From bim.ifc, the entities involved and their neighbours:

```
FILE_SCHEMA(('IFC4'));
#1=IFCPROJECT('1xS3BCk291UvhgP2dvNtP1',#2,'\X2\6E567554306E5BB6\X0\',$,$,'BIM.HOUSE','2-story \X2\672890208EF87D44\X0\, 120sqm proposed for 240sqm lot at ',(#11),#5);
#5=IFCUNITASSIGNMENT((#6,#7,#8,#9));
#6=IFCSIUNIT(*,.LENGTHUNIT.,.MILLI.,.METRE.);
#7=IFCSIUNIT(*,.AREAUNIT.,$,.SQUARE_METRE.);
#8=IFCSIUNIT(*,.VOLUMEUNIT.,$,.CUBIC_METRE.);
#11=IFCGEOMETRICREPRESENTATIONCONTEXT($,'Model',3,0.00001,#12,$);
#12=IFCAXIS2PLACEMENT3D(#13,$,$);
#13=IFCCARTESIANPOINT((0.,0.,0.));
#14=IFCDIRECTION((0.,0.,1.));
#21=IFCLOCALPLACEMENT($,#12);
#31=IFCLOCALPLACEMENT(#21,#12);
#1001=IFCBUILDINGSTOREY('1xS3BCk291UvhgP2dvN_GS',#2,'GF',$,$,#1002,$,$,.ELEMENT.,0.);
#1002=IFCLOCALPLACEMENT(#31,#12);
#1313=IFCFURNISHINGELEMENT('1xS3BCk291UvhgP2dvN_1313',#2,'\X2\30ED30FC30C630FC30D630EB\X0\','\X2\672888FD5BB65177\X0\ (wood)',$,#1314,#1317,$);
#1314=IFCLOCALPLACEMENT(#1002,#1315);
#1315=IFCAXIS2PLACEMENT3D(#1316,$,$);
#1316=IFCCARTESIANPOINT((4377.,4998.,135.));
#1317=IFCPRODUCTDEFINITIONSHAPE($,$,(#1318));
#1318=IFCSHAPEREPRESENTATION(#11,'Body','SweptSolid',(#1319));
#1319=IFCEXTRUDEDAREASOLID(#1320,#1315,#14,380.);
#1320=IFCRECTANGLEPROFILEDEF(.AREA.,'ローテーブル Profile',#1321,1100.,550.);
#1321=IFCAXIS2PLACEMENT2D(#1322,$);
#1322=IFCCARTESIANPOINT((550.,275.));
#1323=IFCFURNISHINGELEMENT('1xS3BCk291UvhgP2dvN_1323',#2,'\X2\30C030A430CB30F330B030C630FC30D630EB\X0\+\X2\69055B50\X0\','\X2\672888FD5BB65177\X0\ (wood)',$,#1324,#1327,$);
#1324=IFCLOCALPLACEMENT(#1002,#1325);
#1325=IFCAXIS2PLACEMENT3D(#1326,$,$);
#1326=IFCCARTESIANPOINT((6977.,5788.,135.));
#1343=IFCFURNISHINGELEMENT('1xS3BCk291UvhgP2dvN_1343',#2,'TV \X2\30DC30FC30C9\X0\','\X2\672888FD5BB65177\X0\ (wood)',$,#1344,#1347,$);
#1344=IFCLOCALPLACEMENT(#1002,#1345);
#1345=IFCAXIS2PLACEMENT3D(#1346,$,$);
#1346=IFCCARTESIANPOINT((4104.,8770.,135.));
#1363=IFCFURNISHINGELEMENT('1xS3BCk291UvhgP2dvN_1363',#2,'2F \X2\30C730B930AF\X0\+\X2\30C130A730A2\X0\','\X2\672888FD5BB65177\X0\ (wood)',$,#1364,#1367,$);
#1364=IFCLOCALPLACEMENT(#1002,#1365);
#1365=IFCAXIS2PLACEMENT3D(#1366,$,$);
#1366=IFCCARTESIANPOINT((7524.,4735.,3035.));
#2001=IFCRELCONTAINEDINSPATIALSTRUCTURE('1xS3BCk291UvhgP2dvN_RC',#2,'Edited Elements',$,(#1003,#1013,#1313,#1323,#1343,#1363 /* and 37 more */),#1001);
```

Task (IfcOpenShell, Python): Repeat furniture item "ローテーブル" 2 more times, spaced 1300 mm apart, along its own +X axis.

```python
import ifcopenshell
import ifcopenshell.api.geometry
import ifcopenshell.api.root
import ifcopenshell.util.element
import ifcopenshell.util.placement
import ifcopenshell.util.unit

model = ifcopenshell.open("bim.ifc")
unit_scale = ifcopenshell.util.unit.calculate_unit_scale(model)


def reuse_history(source, copy):
    """copy_class also copies each property set's owner history, people and application; keep the originals."""
    for rel in copy.IsDefinedBy:
        if rel.is_a("IfcRelDefinesByProperties") and (history := rel.RelatingPropertyDefinition.OwnerHistory):
            rel.RelatingPropertyDefinition.OwnerHistory = source.OwnerHistory
            ifcopenshell.util.element.remove_deep2(model, history)


source = model.by_guid("1xS3BCk291UvhgP2dvN_1313")
base = ifcopenshell.util.placement.get_local_placement(source.ObjectPlacement)
step = base[:3, 0] * 1.3 / unit_scale

for i in range(1, 3):
    copy = ifcopenshell.api.root.copy_class(model, product=source)
    copy.Representation = ifcopenshell.util.element.copy_deep(
        model, source.Representation, exclude=["IfcGeometricRepresentationContext", "IfcRepresentationMap"]
    )
    reuse_history(source, copy)
    matrix = base.copy()
    matrix[:3, 3] += i * step
    print("added at", matrix[:3, 3].round(3) + 0.0)
    ifcopenshell.api.geometry.edit_object_placement(model, product=copy, matrix=matrix, is_si=False)

model.write("bim-out.ifc")
```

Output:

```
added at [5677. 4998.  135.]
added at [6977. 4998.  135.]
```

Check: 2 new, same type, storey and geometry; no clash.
